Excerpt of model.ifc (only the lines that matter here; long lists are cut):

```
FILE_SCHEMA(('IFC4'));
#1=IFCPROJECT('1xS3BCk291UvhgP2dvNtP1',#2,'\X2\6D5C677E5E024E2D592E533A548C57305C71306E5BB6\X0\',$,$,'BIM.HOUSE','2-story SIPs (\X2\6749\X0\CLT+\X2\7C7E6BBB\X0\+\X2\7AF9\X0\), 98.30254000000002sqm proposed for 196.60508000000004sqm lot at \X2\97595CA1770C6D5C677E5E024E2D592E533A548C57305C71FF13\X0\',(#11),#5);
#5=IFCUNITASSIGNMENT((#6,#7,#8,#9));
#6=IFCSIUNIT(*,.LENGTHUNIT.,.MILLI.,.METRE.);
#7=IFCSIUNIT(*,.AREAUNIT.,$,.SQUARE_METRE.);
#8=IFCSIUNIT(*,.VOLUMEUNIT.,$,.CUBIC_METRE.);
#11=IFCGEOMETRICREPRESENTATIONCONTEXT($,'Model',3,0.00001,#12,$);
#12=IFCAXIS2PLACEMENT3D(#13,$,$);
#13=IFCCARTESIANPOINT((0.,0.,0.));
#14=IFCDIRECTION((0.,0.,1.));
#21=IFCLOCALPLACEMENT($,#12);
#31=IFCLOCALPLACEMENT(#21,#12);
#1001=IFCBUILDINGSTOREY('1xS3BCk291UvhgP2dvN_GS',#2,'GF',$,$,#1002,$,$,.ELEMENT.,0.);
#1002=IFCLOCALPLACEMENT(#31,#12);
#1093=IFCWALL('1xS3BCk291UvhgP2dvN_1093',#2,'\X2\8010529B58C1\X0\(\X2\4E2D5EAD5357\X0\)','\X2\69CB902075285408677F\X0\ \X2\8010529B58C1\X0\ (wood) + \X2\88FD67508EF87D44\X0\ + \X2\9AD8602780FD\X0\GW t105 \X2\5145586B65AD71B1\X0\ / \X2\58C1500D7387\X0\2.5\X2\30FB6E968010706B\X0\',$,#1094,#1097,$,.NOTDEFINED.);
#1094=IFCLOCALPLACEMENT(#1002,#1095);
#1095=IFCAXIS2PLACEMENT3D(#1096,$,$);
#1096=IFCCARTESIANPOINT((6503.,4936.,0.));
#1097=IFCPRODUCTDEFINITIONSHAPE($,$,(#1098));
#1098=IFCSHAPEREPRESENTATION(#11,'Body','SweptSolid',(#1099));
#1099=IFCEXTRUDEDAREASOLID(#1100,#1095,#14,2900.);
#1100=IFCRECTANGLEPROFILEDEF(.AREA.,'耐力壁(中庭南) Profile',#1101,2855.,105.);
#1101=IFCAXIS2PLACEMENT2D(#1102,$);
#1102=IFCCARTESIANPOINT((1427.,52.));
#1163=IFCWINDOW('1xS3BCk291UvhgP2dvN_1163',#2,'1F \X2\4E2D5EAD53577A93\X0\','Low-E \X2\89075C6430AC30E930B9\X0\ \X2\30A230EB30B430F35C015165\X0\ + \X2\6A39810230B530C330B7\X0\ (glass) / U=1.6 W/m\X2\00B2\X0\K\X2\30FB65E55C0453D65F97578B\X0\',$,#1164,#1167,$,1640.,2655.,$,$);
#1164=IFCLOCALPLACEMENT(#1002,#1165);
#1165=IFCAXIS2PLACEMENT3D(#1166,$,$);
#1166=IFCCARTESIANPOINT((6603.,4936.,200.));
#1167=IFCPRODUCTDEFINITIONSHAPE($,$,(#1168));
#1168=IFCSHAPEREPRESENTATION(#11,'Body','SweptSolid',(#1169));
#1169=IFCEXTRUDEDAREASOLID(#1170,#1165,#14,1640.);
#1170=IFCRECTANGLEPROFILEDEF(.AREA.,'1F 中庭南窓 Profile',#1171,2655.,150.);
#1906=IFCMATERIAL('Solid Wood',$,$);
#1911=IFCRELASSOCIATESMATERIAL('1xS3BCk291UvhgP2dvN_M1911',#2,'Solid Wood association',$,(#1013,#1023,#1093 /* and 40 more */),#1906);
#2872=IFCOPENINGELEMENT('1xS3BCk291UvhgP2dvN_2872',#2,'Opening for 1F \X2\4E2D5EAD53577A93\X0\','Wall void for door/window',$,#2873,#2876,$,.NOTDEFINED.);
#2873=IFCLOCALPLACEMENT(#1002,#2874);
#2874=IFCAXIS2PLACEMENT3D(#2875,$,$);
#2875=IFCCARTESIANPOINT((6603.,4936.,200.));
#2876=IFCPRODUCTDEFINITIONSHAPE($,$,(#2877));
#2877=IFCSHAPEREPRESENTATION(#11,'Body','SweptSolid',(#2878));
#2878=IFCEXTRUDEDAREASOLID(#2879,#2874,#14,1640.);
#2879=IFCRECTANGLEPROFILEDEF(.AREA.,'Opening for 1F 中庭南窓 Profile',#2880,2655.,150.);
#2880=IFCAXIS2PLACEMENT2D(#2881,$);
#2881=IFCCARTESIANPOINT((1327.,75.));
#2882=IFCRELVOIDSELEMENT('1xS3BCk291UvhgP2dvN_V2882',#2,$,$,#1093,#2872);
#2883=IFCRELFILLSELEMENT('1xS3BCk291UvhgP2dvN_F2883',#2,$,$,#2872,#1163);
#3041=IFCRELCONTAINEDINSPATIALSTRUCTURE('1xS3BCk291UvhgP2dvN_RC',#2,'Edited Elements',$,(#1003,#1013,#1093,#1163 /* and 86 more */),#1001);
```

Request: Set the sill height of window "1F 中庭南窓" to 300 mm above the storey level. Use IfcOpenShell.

```python
import numpy as np
import ifcopenshell
import ifcopenshell.api.geometry
import ifcopenshell.geom
import ifcopenshell.util.element
import ifcopenshell.util.placement
import ifcopenshell.util.shape
import ifcopenshell.util.unit

model = ifcopenshell.open("model.ifc")
unit_scale = ifcopenshell.util.unit.calculate_unit_scale(model)

window = model.by_id(1163)
opening = window.FillsVoids[0].RelatingOpeningElement
storey = ifcopenshell.util.element.get_container(window, ifc_class="IfcBuildingStorey")
level = ifcopenshell.util.placement.get_local_placement(storey.ObjectPlacement)[2, 3]

# The opening's origin need not be at the sill, so measure its lowest point.
shape = ifcopenshell.geom.create_shape(ifcopenshell.geom.settings(), opening)
bottom = ifcopenshell.util.shape.get_shape_bottom_elevation(shape, shape.geometry) / unit_scale
dz = level + 300.0 - bottom

shift = np.array([0.0, 0.0, dz])
# The window is not placed relative to its opening, so move both.
for product in (opening, window):
    matrix = ifcopenshell.util.placement.get_local_placement(product.ObjectPlacement)
    matrix[:3, 3] += shift
    ifcopenshell.api.geometry.edit_object_placement(model, product=product, matrix=matrix, is_si=False)

print(f"moved by {dz * unit_scale:+.3f} m")

model.write("model_updated.ifc")
```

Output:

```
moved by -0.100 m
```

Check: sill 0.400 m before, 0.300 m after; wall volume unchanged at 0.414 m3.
